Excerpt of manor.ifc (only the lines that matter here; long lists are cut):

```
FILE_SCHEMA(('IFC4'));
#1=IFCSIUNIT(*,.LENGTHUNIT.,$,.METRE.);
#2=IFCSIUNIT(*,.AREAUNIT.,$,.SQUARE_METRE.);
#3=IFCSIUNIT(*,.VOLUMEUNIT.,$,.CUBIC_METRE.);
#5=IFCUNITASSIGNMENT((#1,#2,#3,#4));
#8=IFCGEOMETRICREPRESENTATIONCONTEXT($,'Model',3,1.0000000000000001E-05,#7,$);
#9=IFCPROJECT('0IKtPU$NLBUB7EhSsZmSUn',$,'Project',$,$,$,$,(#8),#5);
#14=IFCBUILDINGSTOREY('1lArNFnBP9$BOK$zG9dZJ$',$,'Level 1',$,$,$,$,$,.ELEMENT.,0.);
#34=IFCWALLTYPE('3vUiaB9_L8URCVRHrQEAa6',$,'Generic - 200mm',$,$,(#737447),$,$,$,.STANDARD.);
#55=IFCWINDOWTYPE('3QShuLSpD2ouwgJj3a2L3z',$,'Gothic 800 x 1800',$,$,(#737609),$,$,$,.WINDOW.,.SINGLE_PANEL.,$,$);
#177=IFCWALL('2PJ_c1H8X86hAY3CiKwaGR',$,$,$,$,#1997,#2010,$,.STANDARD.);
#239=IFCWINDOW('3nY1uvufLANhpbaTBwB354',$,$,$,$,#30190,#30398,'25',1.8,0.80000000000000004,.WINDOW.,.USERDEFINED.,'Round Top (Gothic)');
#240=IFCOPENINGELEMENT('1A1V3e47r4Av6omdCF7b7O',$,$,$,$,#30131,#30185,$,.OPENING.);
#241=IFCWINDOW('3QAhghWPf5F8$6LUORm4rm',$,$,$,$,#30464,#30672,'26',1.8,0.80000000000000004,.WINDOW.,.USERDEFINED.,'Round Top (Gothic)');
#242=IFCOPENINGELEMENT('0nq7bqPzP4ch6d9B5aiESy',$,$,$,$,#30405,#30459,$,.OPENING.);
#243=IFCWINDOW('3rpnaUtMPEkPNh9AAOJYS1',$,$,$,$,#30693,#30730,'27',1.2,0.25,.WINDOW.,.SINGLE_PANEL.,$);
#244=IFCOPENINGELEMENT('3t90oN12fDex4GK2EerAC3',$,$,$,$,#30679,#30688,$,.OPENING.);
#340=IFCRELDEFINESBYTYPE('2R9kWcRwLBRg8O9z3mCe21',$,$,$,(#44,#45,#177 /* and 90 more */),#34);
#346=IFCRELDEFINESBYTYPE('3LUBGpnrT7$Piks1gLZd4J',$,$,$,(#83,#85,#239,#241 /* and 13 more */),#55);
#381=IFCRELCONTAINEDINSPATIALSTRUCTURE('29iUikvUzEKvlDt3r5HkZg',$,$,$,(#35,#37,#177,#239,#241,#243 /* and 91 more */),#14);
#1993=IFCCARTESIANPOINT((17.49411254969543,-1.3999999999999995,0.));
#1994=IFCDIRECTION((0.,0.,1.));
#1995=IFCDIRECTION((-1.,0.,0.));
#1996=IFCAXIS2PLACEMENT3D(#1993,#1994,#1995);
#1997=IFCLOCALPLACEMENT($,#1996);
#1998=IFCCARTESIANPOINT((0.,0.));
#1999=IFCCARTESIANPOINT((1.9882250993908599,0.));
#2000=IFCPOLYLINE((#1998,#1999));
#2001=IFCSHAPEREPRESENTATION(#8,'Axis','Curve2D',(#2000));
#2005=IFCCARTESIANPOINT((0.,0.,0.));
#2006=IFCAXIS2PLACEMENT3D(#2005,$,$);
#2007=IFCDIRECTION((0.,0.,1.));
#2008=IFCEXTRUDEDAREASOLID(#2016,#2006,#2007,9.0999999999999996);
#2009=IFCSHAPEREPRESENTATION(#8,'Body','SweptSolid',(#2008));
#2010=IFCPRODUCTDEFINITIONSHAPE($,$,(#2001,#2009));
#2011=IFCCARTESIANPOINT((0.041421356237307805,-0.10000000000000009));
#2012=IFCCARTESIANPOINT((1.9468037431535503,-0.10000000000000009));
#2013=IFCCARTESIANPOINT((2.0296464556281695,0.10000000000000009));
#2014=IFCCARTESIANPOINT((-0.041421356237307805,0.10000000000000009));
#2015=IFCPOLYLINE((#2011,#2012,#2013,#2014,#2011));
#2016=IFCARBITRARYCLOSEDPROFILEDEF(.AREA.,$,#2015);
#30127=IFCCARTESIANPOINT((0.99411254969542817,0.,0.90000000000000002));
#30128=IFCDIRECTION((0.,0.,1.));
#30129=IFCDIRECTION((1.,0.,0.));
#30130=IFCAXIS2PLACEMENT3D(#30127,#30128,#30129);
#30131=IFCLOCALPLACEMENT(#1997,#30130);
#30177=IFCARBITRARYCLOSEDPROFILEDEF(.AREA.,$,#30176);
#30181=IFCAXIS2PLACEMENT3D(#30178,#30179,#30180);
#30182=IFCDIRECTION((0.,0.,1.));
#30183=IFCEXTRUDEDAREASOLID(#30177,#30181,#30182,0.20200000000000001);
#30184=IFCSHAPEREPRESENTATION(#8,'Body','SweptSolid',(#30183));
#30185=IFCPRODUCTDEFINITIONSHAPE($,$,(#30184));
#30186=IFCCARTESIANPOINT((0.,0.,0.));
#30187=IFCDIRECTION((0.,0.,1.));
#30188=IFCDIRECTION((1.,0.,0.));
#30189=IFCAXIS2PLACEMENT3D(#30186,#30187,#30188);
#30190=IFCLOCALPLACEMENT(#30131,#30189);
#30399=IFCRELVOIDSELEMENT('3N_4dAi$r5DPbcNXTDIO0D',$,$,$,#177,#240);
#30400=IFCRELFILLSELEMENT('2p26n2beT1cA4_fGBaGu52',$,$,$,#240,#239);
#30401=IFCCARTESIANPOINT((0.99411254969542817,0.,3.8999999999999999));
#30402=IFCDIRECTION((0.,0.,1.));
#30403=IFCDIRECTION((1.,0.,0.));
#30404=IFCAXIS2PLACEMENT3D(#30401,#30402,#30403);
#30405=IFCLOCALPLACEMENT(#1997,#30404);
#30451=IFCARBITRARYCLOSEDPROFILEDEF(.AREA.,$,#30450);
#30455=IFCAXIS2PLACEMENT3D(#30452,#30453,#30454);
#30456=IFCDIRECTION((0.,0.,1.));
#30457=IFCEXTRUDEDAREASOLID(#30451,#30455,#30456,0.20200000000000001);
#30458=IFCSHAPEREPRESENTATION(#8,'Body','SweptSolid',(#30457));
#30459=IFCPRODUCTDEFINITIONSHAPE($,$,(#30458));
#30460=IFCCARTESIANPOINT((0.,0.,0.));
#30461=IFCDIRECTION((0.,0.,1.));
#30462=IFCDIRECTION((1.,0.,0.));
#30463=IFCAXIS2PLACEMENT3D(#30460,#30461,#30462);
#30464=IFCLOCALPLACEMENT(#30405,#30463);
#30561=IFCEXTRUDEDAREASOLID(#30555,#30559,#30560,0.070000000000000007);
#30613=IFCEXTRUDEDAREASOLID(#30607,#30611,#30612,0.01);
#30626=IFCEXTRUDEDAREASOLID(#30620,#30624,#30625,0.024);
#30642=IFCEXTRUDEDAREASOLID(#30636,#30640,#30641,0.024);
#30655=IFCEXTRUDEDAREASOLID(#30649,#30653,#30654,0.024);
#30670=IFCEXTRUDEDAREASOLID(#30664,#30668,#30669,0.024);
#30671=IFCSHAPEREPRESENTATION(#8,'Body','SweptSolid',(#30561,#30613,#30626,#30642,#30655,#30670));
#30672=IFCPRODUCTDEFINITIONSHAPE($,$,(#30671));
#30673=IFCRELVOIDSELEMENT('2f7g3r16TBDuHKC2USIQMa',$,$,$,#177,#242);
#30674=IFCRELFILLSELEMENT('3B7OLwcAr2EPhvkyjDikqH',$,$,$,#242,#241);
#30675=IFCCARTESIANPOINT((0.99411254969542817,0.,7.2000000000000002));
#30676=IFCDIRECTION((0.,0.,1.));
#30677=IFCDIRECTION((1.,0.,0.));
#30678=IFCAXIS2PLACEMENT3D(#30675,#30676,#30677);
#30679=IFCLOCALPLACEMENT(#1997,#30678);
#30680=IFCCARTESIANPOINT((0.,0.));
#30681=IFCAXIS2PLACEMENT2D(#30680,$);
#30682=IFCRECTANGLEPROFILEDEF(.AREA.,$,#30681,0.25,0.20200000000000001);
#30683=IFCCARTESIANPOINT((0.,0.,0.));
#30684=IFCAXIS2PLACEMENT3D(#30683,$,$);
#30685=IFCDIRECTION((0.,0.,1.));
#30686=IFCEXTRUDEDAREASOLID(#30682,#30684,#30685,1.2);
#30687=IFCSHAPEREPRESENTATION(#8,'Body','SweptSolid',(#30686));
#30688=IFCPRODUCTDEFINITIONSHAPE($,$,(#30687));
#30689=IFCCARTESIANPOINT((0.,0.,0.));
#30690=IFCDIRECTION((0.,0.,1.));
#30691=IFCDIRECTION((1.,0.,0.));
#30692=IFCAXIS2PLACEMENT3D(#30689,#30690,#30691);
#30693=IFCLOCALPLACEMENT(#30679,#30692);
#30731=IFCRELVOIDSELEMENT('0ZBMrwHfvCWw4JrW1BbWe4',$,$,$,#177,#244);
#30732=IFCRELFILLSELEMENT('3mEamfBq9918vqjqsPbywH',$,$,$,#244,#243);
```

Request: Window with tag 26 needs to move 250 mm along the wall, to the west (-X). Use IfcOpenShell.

```python
import ifcopenshell
import ifcopenshell.api.geometry
import ifcopenshell.util.placement

model = ifcopenshell.open("manor.ifc")

window = model.by_guid("3QAhghWPf5F8$6LUORm4rm")
opening = window.FillsVoids[0].RelatingOpeningElement
wall = opening.VoidsElements[0].RelatingBuildingElement

wall_matrix = ifcopenshell.util.placement.get_local_placement(wall.ObjectPlacement)
shift = wall_matrix[:3, 0] * 0.25
before = ifcopenshell.util.placement.get_local_placement(window.ObjectPlacement)[:3, 3].copy()

# The window is placed relative to its opening, so it follows when the opening moves.
matrix = ifcopenshell.util.placement.get_local_placement(opening.ObjectPlacement)
matrix[:3, 3] += shift
ifcopenshell.api.geometry.edit_object_placement(
    model, product=opening, matrix=matrix, is_si=False, should_transform_children=True
)

after = ifcopenshell.util.placement.get_local_placement(window.ObjectPlacement)[:3, 3]
print("window moved by", (after - before).round(3) + 0.0)

model.write("manor-out.ifc")
```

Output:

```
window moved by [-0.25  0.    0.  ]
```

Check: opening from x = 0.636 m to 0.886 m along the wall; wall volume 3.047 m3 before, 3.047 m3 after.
